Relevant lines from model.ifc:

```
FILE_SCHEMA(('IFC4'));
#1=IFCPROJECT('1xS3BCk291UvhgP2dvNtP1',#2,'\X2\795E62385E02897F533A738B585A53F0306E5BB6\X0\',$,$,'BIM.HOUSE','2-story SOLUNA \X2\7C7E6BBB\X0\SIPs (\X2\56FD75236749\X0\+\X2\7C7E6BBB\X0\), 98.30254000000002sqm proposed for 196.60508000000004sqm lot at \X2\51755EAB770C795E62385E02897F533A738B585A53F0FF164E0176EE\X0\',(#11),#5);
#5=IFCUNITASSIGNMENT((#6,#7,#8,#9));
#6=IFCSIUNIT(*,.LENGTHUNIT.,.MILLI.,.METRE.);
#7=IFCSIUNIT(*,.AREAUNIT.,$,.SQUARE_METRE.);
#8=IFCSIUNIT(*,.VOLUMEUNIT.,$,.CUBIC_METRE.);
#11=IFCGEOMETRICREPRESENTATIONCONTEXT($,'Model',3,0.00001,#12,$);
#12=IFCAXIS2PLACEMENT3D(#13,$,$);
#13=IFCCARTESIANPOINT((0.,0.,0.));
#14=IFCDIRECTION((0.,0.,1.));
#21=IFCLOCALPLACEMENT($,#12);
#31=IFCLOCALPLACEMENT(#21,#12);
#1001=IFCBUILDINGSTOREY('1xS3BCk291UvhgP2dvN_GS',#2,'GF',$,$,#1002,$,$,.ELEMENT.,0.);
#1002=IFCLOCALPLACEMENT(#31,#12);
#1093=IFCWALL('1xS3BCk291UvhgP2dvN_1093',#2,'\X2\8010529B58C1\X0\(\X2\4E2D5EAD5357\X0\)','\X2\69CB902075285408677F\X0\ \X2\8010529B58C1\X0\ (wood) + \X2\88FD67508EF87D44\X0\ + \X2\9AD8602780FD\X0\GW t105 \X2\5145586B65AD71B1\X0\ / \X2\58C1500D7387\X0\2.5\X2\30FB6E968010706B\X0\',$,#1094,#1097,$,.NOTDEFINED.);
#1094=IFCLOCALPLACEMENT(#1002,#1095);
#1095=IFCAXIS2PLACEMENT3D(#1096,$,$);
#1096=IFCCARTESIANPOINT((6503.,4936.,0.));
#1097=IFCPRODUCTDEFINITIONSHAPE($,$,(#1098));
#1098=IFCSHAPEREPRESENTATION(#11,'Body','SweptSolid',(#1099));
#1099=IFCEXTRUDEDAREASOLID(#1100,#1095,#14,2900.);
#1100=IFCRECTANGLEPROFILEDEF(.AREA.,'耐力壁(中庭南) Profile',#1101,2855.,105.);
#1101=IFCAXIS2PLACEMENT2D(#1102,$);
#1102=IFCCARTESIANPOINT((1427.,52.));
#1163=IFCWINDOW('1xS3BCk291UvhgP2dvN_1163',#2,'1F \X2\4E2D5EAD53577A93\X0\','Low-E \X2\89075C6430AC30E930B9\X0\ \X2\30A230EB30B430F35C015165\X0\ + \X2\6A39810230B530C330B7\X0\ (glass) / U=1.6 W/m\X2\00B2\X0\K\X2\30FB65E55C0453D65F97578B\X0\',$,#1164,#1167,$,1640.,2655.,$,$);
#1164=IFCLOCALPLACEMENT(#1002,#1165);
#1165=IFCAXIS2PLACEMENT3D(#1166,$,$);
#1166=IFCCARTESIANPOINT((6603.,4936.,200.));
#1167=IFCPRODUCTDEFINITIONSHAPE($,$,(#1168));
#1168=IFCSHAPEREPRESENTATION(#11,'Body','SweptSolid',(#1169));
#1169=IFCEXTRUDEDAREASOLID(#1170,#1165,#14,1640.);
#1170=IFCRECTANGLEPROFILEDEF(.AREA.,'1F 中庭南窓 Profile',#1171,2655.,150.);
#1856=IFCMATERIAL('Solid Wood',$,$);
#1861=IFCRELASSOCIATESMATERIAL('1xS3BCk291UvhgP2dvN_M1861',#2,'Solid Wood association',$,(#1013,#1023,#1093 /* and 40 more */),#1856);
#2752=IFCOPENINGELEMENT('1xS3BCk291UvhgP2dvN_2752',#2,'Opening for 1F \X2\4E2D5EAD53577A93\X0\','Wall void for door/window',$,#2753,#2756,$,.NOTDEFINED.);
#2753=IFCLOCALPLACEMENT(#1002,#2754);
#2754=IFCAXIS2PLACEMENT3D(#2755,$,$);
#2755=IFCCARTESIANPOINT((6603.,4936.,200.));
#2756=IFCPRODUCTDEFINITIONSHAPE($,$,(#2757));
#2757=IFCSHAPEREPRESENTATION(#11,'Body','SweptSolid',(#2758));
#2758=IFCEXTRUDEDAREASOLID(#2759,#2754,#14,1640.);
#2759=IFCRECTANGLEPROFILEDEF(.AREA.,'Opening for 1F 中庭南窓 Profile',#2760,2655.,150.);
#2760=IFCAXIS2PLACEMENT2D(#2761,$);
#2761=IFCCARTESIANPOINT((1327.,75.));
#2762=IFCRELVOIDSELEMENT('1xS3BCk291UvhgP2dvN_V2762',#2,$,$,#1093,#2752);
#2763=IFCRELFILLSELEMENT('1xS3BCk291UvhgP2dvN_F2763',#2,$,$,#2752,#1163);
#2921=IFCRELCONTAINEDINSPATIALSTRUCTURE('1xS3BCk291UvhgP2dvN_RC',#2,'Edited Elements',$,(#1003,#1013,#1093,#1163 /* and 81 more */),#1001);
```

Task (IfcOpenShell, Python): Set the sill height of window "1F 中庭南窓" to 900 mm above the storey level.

```python
import numpy as np
import ifcopenshell
import ifcopenshell.api.geometry
import ifcopenshell.geom
import ifcopenshell.util.element
import ifcopenshell.util.placement
import ifcopenshell.util.shape
import ifcopenshell.util.unit

model = ifcopenshell.open("model.ifc")
unit_scale = ifcopenshell.util.unit.calculate_unit_scale(model)

window = model.by_guid("1xS3BCk291UvhgP2dvN_1163")
opening = window.FillsVoids[0].RelatingOpeningElement
storey = ifcopenshell.util.element.get_container(window, ifc_class="IfcBuildingStorey")
level = ifcopenshell.util.placement.get_local_placement(storey.ObjectPlacement)[2, 3]

# The opening's origin need not be at the sill, so measure its lowest point.
shape = ifcopenshell.geom.create_shape(ifcopenshell.geom.settings(), opening)
bottom = ifcopenshell.util.shape.get_shape_bottom_elevation(shape, shape.geometry) / unit_scale
dz = level + 900.0 - bottom

shift = np.array([0.0, 0.0, dz])
# The window is not placed relative to its opening, so move both.
for product in (opening, window):
    matrix = ifcopenshell.util.placement.get_local_placement(product.ObjectPlacement)
    matrix[:3, 3] += shift
    ifcopenshell.api.geometry.edit_object_placement(model, product=product, matrix=matrix, is_si=False)

print(f"moved by {dz * unit_scale:+.3f} m")

model.write("model-out.ifc")
```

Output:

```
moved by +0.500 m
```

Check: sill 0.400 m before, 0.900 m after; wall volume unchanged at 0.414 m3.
